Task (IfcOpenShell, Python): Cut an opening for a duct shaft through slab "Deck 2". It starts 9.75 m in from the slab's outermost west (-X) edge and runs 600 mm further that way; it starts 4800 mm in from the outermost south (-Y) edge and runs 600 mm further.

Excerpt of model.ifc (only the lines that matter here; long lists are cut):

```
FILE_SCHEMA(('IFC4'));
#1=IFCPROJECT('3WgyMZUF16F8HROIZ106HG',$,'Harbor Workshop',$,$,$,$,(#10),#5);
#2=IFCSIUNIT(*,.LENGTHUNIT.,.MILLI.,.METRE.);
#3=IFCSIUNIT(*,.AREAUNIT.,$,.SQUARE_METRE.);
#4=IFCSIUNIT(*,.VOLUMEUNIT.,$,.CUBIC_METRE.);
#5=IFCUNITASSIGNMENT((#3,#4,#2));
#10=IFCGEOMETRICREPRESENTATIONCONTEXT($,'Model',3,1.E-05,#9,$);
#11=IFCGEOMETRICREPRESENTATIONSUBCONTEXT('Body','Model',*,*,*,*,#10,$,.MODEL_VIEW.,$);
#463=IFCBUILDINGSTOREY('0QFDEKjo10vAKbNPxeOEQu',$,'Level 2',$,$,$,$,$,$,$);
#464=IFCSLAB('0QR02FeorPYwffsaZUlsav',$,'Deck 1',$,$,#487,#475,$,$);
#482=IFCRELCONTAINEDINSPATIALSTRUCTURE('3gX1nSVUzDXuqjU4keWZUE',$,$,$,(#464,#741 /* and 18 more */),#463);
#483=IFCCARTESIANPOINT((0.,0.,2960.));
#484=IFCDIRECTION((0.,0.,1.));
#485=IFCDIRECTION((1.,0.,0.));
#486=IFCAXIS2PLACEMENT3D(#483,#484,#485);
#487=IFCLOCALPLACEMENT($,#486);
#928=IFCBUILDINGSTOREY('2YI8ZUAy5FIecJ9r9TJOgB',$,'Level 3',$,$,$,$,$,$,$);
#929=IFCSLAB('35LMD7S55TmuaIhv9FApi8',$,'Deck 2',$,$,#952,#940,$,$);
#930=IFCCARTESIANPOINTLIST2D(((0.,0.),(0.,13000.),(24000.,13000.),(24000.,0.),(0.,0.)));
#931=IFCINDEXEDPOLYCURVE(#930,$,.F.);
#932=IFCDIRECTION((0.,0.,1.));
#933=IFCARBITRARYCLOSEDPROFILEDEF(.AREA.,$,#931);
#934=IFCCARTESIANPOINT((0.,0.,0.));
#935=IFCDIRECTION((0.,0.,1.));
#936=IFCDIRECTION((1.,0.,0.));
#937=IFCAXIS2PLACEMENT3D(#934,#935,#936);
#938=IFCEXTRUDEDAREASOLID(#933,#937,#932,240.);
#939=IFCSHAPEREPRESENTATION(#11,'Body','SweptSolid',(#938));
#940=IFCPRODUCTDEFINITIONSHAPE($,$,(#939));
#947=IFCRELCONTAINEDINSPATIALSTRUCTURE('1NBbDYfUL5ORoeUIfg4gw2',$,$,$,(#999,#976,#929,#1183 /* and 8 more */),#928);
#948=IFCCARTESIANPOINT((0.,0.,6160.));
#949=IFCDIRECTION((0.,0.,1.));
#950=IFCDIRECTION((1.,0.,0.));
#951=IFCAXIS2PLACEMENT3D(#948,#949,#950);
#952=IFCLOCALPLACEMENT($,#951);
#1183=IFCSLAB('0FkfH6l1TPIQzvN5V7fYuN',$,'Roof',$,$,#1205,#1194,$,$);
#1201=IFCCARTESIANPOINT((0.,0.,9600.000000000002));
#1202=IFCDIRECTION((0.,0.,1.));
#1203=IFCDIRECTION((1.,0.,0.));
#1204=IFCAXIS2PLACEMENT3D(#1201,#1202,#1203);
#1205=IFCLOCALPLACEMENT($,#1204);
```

```python
import numpy as np
import ifcopenshell
import ifcopenshell.api.feature
import ifcopenshell.api.geometry
import ifcopenshell.api.root
import ifcopenshell.geom
import ifcopenshell.util.placement
import ifcopenshell.util.representation
import ifcopenshell.util.shape
import ifcopenshell.util.unit

model = ifcopenshell.open("model.ifc")
unit_scale = ifcopenshell.util.unit.calculate_unit_scale(model)
settings = ifcopenshell.geom.settings()


def volume(element):
    """Net volume in cubic metres, openings subtracted."""
    shape = ifcopenshell.geom.create_shape(settings, element)
    return ifcopenshell.util.shape.get_volume(shape.geometry)


slab = model.by_guid("35LMD7S55TmuaIhv9FApi8")
before = volume(slab)

# Extent in the slab's own axes, in metres. The edges named are its -X and -Y sides.
slab_shape = ifcopenshell.geom.create_shape(settings, slab)
vertices = ifcopenshell.util.shape.get_vertices(slab_shape.geometry)
x_min, y_min, bottom = vertices.min(axis=0)
top = vertices[:, 2].max()

opening = ifcopenshell.api.root.create_entity(model, ifc_class="IfcOpeningElement", name="Duct shaft opening", predefined_type="OPENING")
context = ifcopenshell.util.representation.get_context(model, "Model", "Body", "MODEL_VIEW")
width, depth = 0.6, 0.6
outline = [(0.0, 0.0), (width, 0.0), (width, depth), (0.0, depth), (0.0, 0.0)]
# Overshoot both faces by 50 mm so the cut is clean.
shape = ifcopenshell.api.geometry.add_slab_representation(
    model, context=context, depth=top - bottom + 0.1, polyline=outline
)
ifcopenshell.api.geometry.assign_representation(model, product=opening, representation=shape)

matrix = ifcopenshell.util.placement.get_local_placement(slab.ObjectPlacement)
matrix[:, 3] = matrix @ np.append(np.array([x_min + 9.75, y_min + 4.8, bottom - 0.05]) / unit_scale, 1.0)
ifcopenshell.api.geometry.edit_object_placement(model, product=opening, matrix=matrix, is_si=False)
ifcopenshell.api.feature.add_feature(model, feature=opening, element=slab)

after = volume(slab)

print(f"slab volume {before:.3f} -> {after:.3f} m3")

model.write("model_updated.ifc")
```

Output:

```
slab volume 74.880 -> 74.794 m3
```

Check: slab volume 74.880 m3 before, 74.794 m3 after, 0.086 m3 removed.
